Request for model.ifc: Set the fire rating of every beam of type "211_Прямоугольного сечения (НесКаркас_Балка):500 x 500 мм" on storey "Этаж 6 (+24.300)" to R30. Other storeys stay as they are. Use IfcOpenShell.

First a look at what the model holds.

```python
import ifcopenshell
import ifcopenshell.util.element

model = ifcopenshell.open("model.ifc")
print(model.schema)
storey = next(s for s in model.by_type("IfcBuildingStorey") if s.Name == "Этаж 6 (+24.300)")
beams = [e for e in ifcopenshell.util.element.get_decomposition(storey) if e.is_a("IfcBeam")]
seen = {}
for e in beams:
    element_type = ifcopenshell.util.element.get_type(e)
    key = (element_type.Name if element_type != e and element_type else None, ifcopenshell.util.element.get_pset(e, "Pset_BeamCommon", "FireRating"))
    seen[key] = seen.get(key, 0) + 1
for (name, value), count in sorted(seen.items(), key=str):
    print(count, "x", name, "|", value)
```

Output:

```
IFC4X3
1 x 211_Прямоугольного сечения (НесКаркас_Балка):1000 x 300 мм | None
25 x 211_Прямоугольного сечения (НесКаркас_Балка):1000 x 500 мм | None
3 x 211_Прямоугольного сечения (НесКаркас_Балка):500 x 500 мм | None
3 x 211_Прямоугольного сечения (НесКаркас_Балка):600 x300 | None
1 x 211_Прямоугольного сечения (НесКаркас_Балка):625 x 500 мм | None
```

```python
import ifcopenshell
import ifcopenshell.api.pset
import ifcopenshell.util.element

model = ifcopenshell.open("model.ifc")

storey = next(s for s in model.by_type("IfcBuildingStorey") if s.Name == "Этаж 6 (+24.300)")
beams = [e for e in ifcopenshell.util.element.get_decomposition(storey) if e.is_a("IfcBeam")]

count = 0
for e in beams:
    element_type = ifcopenshell.util.element.get_type(e)
    if element_type in (None, e) or element_type.Name != "211_Прямоугольного сечения (НесКаркас_Балка):500 x 500 мм":
        continue
    # add_pset returns the element's existing set when there is one.
    pset = ifcopenshell.api.pset.add_pset(model, product=e, name="Pset_BeamCommon")
    ifcopenshell.api.pset.edit_pset(model, pset=pset, properties={"FireRating": "R30"})
    count += 1

print(count, "beams updated")

model.write("model_edited.ifc")
```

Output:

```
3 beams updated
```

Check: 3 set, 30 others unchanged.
